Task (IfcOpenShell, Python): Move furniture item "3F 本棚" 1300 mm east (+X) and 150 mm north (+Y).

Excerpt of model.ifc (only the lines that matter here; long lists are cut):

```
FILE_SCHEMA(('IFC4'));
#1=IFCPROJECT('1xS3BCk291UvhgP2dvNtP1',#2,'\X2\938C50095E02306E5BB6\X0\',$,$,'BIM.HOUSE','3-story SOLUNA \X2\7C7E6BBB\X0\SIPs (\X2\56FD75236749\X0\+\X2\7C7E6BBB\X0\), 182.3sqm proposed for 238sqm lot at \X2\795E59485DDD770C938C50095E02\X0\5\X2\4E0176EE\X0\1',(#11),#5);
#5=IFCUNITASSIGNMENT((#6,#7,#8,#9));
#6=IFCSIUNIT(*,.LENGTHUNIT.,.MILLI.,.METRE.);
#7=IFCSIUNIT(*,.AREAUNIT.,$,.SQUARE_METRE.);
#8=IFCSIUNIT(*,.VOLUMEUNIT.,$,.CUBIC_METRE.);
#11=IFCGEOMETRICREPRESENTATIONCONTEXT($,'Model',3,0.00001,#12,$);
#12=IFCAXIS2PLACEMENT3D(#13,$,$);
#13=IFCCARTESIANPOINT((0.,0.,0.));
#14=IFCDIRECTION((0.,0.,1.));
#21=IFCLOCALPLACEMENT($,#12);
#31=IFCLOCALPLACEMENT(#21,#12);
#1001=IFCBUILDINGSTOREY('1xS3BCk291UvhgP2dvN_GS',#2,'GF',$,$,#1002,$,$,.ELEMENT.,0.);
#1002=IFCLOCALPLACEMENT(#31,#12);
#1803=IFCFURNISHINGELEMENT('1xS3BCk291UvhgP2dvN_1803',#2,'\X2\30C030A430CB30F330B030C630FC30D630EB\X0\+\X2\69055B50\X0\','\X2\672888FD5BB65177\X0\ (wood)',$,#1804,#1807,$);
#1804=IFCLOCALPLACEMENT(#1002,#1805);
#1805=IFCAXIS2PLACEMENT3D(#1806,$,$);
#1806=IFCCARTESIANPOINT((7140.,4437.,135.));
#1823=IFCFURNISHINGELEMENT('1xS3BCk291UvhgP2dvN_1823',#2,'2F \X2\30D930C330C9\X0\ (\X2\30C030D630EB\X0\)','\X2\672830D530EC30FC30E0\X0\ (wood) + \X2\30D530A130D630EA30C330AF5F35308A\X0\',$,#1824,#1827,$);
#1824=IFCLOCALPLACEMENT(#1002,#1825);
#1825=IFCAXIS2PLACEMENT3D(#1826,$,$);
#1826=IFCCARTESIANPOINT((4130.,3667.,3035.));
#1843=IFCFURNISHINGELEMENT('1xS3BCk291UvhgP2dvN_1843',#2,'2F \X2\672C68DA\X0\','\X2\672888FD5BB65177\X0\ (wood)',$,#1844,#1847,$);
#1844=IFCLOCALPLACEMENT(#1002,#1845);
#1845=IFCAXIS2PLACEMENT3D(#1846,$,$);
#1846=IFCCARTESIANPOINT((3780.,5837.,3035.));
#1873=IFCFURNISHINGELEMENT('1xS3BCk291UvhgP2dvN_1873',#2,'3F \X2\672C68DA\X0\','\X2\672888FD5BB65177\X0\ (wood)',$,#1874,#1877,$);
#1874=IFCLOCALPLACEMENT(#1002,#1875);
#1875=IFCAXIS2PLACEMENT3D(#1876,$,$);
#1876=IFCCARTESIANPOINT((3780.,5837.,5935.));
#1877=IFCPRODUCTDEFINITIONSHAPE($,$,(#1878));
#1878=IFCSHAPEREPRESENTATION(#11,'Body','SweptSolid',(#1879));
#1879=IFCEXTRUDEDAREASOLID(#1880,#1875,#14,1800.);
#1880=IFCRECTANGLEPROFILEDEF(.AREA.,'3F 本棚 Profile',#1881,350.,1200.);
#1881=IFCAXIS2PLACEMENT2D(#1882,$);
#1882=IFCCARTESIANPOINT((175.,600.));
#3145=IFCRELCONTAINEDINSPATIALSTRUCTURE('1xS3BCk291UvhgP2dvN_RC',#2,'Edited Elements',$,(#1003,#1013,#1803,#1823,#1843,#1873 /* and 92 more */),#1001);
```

```python
import ifcopenshell
import ifcopenshell.api.geometry
import ifcopenshell.util.placement
import ifcopenshell.util.unit

model = ifcopenshell.open("model.ifc")
unit_scale = ifcopenshell.util.unit.calculate_unit_scale(model)

item = model.by_guid("1xS3BCk291UvhgP2dvN_1873")
matrix = ifcopenshell.util.placement.get_local_placement(item.ObjectPlacement)
matrix[0, 3] += 1.3 / unit_scale
matrix[1, 3] += 0.15 / unit_scale
ifcopenshell.api.geometry.edit_object_placement(model, product=item, matrix=matrix, is_si=False)

print(ifcopenshell.util.placement.get_local_placement(item.ObjectPlacement).round(3) + 0.0)

model.write("model_edited.ifc")
```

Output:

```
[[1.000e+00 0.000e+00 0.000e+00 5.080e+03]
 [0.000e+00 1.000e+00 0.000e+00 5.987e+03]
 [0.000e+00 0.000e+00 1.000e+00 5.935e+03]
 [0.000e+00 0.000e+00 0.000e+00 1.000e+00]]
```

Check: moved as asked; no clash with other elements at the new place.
